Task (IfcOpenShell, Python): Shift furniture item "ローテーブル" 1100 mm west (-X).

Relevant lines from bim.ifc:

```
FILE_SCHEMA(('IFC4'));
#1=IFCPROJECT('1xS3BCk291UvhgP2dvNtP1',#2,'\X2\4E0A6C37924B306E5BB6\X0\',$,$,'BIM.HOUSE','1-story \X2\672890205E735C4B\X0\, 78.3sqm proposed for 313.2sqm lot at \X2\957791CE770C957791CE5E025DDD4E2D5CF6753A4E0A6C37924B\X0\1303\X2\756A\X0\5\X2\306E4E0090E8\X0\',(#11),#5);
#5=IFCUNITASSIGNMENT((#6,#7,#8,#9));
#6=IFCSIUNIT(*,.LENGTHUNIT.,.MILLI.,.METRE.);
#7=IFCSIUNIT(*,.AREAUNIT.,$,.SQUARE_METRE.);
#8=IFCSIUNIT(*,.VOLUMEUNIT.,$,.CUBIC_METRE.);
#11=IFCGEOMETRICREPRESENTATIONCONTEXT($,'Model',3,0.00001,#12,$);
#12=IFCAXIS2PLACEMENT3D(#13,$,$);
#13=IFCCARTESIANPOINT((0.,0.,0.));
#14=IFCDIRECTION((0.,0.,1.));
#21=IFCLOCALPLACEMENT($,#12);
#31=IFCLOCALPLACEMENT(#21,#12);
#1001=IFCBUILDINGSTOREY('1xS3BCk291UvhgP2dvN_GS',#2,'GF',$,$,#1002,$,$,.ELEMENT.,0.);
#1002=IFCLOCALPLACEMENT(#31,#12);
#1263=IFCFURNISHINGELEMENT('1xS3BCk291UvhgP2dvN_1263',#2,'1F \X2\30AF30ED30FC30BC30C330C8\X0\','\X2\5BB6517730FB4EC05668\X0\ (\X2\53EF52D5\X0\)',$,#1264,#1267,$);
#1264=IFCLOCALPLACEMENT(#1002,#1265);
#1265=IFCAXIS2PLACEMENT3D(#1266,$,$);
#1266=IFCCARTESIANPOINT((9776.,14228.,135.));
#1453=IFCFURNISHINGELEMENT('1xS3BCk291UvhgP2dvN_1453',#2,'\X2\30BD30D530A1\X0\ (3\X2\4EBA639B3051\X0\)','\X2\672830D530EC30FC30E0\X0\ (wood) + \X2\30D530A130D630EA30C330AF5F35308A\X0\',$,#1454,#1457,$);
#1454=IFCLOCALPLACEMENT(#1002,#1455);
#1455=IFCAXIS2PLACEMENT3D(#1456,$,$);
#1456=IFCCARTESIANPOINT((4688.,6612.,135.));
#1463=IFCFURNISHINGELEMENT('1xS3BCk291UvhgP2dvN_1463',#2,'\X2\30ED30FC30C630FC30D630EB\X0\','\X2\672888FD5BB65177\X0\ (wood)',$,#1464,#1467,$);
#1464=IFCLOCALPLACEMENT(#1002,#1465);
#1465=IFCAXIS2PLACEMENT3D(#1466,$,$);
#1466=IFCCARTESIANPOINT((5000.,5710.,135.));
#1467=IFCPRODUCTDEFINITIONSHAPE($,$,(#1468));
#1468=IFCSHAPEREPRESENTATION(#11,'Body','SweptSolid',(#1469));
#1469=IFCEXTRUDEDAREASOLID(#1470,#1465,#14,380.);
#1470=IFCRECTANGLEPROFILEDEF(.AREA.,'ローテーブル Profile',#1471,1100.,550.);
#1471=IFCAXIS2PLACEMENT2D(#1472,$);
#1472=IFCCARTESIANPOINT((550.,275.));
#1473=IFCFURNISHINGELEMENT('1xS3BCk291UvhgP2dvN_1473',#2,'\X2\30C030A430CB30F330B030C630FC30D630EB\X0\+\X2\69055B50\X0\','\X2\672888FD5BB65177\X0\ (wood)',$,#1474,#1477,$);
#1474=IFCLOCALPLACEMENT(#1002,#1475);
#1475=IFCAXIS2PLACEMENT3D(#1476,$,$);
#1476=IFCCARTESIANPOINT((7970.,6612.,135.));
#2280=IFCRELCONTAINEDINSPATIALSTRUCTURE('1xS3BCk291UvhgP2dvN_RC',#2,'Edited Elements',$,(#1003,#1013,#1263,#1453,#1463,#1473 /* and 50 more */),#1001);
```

```python
import ifcopenshell
import ifcopenshell.api.geometry
import ifcopenshell.util.placement

model = ifcopenshell.open("bim.ifc")

item = model.by_guid("1xS3BCk291UvhgP2dvN_1463")
matrix = ifcopenshell.util.placement.get_local_placement(item.ObjectPlacement)
matrix[0, 3] -= 1100.0
ifcopenshell.api.geometry.edit_object_placement(model, product=item, matrix=matrix, is_si=False)

print(ifcopenshell.util.placement.get_local_placement(item.ObjectPlacement).round(3) + 0.0)

model.write("bim-out.ifc")
```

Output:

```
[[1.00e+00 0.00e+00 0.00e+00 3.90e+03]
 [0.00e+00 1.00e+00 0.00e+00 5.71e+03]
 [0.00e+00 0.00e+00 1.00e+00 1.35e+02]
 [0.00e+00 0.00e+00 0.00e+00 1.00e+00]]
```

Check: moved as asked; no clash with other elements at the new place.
